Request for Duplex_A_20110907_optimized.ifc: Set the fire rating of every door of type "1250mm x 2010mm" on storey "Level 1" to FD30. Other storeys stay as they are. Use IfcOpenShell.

First a look at what the model holds.

```python
import ifcopenshell
import ifcopenshell.util.element

model = ifcopenshell.open("Duplex_A_20110907_optimized.ifc")
print(model.schema)
storey = next(s for s in model.by_type("IfcBuildingStorey") if s.Name == "Level 1")
doors = [e for e in ifcopenshell.util.element.get_decomposition(storey) if e.is_a("IfcDoor")]
seen = {}
for e in doors:
    element_type = ifcopenshell.util.element.get_type(e)
    key = (element_type.Name if element_type != e and element_type else None, ifcopenshell.util.element.get_pset(e, "Pset_DoorCommon", "FireRating"))
    seen[key] = seen.get(key, 0) + 1
for (name, value), count in sorted(seen.items(), key=str):
    print(count, "x", name, "|", value)
```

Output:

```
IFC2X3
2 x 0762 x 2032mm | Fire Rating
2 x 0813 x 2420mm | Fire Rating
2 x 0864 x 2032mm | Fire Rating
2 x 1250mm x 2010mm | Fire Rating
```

```python
import ifcopenshell
import ifcopenshell.api.pset
import ifcopenshell.util.element

model = ifcopenshell.open("Duplex_A_20110907_optimized.ifc")

storey = next(s for s in model.by_type("IfcBuildingStorey") if s.Name == "Level 1")
doors = [e for e in ifcopenshell.util.element.get_decomposition(storey) if e.is_a("IfcDoor")]

count = 0
for e in doors:
    element_type = ifcopenshell.util.element.get_type(e)
    if element_type in (None, e) or element_type.Name != "1250mm x 2010mm":
        continue
    # add_pset returns the element's existing set when there is one.
    pset = ifcopenshell.api.pset.add_pset(model, product=e, name="Pset_DoorCommon")
    ifcopenshell.api.pset.edit_pset(model, pset=pset, properties={"FireRating": "FD30"})
    count += 1

print(count, "doors updated")

model.write("Duplex_A_20110907_optimized_rev.ifc")
```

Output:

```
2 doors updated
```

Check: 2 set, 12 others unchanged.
